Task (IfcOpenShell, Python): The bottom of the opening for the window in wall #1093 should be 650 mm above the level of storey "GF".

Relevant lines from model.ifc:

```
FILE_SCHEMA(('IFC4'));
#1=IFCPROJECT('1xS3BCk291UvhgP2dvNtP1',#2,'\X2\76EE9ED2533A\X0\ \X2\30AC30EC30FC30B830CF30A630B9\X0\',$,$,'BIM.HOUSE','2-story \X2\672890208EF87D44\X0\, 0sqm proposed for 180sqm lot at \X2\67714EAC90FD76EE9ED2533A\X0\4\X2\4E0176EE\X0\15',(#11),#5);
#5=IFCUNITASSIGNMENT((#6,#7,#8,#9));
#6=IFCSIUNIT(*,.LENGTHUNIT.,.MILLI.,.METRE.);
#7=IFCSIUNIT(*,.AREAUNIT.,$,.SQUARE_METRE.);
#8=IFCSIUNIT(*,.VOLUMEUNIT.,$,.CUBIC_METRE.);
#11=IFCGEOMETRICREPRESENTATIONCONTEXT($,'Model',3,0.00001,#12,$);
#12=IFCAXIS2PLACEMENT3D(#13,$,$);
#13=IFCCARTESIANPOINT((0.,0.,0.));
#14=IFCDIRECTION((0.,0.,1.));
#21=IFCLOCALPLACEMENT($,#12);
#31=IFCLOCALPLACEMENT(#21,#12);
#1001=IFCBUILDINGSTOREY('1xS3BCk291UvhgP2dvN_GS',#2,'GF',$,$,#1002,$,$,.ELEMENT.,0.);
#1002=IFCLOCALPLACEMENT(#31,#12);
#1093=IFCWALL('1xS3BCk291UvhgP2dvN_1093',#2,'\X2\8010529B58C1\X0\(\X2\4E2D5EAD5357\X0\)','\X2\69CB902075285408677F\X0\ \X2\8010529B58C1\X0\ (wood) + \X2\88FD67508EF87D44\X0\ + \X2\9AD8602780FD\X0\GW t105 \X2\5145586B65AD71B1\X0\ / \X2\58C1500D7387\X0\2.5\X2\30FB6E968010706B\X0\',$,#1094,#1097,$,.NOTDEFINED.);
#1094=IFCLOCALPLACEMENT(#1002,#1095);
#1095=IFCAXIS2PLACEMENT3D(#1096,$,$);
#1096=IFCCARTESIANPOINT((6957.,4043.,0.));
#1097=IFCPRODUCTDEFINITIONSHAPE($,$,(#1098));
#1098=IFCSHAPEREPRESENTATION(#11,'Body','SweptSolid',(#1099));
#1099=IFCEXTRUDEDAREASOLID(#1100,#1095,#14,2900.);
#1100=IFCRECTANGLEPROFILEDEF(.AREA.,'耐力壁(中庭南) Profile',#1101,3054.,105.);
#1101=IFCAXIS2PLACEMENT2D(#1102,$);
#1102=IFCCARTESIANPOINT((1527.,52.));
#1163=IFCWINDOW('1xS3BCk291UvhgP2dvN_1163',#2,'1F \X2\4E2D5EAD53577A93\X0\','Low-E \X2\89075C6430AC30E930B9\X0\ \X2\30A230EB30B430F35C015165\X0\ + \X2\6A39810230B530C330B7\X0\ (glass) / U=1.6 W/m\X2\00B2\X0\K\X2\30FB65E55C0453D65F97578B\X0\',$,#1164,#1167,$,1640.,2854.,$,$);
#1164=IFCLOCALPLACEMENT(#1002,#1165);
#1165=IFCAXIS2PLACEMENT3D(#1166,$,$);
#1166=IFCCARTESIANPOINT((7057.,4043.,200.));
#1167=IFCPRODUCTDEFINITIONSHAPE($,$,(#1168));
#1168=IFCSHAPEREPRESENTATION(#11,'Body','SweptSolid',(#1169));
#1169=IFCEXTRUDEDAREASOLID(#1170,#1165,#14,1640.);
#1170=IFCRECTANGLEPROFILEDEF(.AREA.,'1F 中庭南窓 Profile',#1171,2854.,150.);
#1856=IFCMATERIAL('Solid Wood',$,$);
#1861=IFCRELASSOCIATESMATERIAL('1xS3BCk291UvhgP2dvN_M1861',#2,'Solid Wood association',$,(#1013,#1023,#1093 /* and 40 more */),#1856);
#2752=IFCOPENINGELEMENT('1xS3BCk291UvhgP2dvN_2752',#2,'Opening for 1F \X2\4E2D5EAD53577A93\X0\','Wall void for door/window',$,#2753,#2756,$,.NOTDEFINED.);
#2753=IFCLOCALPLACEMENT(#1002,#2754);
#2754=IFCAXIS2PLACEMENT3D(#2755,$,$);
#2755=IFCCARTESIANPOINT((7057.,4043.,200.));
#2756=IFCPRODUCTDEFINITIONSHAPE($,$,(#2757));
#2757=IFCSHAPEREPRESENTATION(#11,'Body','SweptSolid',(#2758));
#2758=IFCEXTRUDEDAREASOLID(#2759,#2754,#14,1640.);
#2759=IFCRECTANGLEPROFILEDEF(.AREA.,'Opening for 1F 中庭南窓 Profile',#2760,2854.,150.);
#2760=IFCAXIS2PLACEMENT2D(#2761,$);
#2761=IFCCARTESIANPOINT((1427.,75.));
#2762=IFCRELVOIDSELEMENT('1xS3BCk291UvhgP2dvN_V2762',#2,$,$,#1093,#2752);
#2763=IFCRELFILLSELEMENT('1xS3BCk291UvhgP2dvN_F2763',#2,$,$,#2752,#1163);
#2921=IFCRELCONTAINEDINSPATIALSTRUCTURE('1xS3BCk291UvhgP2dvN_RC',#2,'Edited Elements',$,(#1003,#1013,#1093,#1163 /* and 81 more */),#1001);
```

```python
import numpy as np
import ifcopenshell
import ifcopenshell.api.geometry
import ifcopenshell.geom
import ifcopenshell.util.element
import ifcopenshell.util.placement
import ifcopenshell.util.shape
import ifcopenshell.util.unit

model = ifcopenshell.open("model.ifc")
unit_scale = ifcopenshell.util.unit.calculate_unit_scale(model)

window = model.by_id(1163)
opening = window.FillsVoids[0].RelatingOpeningElement
storey = ifcopenshell.util.element.get_container(window, ifc_class="IfcBuildingStorey")
level = ifcopenshell.util.placement.get_local_placement(storey.ObjectPlacement)[2, 3]

# The opening's origin need not be at the sill, so measure its lowest point.
shape = ifcopenshell.geom.create_shape(ifcopenshell.geom.settings(), opening)
bottom = ifcopenshell.util.shape.get_shape_bottom_elevation(shape, shape.geometry) / unit_scale
dz = level + 0.65 / unit_scale - bottom

shift = np.array([0.0, 0.0, dz])
# The window is not placed relative to its opening, so move both.
for product in (opening, window):
    matrix = ifcopenshell.util.placement.get_local_placement(product.ObjectPlacement)
    matrix[:3, 3] += shift
    ifcopenshell.api.geometry.edit_object_placement(model, product=product, matrix=matrix, is_si=False)

print(f"moved by {dz * unit_scale:+.3f} m")

model.write("model-out.ifc")
```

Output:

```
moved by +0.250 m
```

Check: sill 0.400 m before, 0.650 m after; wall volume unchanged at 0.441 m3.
